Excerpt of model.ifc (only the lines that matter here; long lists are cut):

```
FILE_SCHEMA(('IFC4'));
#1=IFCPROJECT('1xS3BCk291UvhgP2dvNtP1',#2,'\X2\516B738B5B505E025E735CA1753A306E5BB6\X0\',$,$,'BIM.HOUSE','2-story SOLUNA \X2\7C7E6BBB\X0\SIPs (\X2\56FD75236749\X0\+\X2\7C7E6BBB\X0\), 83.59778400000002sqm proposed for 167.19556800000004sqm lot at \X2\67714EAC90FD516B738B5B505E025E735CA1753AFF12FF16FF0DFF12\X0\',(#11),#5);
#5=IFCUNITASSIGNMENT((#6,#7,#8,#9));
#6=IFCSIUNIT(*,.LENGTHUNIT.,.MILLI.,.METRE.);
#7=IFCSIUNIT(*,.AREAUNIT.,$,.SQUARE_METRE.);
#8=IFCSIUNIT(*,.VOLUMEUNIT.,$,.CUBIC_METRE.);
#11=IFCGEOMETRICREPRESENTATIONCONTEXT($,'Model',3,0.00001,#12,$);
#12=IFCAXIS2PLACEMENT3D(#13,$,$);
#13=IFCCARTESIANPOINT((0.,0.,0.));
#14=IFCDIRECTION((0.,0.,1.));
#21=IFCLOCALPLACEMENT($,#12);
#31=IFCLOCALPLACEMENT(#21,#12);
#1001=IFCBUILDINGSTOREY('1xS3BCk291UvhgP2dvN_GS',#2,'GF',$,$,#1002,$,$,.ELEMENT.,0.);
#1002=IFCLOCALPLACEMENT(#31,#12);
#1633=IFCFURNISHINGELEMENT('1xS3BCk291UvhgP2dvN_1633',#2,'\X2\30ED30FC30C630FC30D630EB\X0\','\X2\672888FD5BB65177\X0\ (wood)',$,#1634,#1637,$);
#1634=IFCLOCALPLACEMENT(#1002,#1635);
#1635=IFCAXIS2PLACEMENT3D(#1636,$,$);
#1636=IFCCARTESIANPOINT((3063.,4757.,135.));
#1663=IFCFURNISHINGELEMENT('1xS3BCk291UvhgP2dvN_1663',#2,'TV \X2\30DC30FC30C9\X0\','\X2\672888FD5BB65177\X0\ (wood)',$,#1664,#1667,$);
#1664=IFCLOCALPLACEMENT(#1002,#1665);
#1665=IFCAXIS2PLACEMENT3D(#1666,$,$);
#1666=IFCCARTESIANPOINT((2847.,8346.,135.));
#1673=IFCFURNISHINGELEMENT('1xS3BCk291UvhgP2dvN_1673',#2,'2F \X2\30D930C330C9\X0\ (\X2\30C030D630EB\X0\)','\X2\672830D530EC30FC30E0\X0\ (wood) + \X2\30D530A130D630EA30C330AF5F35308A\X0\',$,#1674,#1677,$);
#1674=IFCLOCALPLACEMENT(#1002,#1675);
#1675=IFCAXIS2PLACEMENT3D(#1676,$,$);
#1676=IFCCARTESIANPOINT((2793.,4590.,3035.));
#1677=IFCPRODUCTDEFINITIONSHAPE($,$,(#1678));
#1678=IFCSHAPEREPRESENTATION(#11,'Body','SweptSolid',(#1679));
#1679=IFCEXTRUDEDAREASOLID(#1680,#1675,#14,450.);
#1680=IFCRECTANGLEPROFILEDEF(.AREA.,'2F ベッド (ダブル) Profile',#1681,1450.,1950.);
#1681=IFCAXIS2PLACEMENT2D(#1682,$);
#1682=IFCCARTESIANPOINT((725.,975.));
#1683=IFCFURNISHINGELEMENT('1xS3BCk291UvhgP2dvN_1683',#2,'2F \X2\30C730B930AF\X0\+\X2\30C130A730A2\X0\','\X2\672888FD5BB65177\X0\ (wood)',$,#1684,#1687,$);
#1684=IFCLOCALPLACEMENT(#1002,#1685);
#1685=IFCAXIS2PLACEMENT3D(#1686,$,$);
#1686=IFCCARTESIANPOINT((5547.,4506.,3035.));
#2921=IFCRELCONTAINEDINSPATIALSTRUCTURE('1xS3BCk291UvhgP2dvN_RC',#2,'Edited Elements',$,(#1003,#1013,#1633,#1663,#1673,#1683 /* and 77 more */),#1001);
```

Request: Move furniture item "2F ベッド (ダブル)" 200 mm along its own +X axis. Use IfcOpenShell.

```python
import ifcopenshell
import ifcopenshell.api.geometry
import ifcopenshell.util.placement

model = ifcopenshell.open("model.ifc")

item = model.by_guid("1xS3BCk291UvhgP2dvN_1673")
matrix = ifcopenshell.util.placement.get_local_placement(item.ObjectPlacement)
matrix[:3, 3] += matrix[:3, 0] * 200.0
ifcopenshell.api.geometry.edit_object_placement(model, product=item, matrix=matrix, is_si=False)

print(ifcopenshell.util.placement.get_local_placement(item.ObjectPlacement).round(3) + 0.0)

model.write("model_v2.ifc")
```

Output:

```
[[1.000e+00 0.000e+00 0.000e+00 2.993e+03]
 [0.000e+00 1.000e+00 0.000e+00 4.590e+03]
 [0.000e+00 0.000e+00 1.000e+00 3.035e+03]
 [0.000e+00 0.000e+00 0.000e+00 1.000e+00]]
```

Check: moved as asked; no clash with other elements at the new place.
